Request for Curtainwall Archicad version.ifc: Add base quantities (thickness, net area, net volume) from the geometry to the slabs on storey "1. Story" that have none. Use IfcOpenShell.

First a look at what the model holds.

```python
import ifcopenshell
import ifcopenshell.util.element
import ifcopenshell.util.unit

model = ifcopenshell.open("Curtainwall Archicad version.ifc")
print(model.schema)
for unit_type in ("LENGTHUNIT", "AREAUNIT", "VOLUMEUNIT"):
    print(unit_type, ifcopenshell.util.unit.calculate_unit_scale(model, unit_type))
storey = next(s for s in model.by_type("IfcBuildingStorey") if s.Name == "1. Story")
slabs = [e for e in ifcopenshell.util.element.get_decomposition(storey) if e.is_a("IfcSlab")]
for e in sorted(slabs, key=lambda e: e.id()):
    print(e.id(), e.is_a(), e.Name, list(ifcopenshell.util.element.get_psets(e, qtos_only=True)), sep=" | ")
```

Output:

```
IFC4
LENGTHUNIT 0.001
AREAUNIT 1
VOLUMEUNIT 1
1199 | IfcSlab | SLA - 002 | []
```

```python
import ifcopenshell
import ifcopenshell.api.pset
import ifcopenshell.geom
import ifcopenshell.util.element
import ifcopenshell.util.shape
import ifcopenshell.util.unit

model = ifcopenshell.open("Curtainwall Archicad version.ifc")
unit_scale = ifcopenshell.util.unit.calculate_unit_scale(model)
area_scale = ifcopenshell.util.unit.calculate_unit_scale(model, "AREAUNIT")
volume_scale = ifcopenshell.util.unit.calculate_unit_scale(model, "VOLUMEUNIT")
settings = ifcopenshell.geom.settings()

storey = next(s for s in model.by_type("IfcBuildingStorey") if s.Name == "1. Story")
slabs = [e for e in ifcopenshell.util.element.get_decomposition(storey) if e.is_a("IfcSlab")]

for e in sorted(slabs, key=lambda e: e.id()):
    if ifcopenshell.util.element.get_psets(e, qtos_only=True, should_inherit=False):
        continue
    # Geometry comes back in metres, in the element's own axes.
    shape = ifcopenshell.geom.create_shape(settings, e)
    values = {
        "Width": ifcopenshell.util.shape.get_z(shape.geometry) / unit_scale,
        "NetArea": ifcopenshell.util.shape.get_footprint_area(shape.geometry) / area_scale,
        "NetVolume": ifcopenshell.util.shape.get_volume(shape.geometry) / volume_scale,
    }
    qto = ifcopenshell.api.pset.add_qto(model, product=e, name="Qto_SlabBaseQuantities")
    ifcopenshell.api.pset.edit_qto(model, qto=qto, properties=values)
    print(e.id(), {k: round(v, 3) for k, v in values.items()})

model.write("Curtainwall Archicad version_rev.ifc")
```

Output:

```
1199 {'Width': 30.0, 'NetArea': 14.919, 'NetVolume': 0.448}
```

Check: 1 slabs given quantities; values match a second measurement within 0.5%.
